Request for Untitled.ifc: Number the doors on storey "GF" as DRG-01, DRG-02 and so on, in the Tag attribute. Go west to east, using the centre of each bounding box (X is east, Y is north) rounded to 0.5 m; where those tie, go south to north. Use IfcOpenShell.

First a look at what the model holds.

```python
import ifcopenshell
import ifcopenshell.util.element
import ifcopenshell.util.placement

model = ifcopenshell.open("Untitled.ifc")
print(model.schema)
storey = next(s for s in model.by_type("IfcBuildingStorey") if s.Name == "GF")
doors = [e for e in ifcopenshell.util.element.get_decomposition(storey) if e.is_a("IfcDoor")]
for e in sorted(doors, key=lambda e: e.id()):
    origin = ifcopenshell.util.placement.get_local_placement(e.ObjectPlacement)[:3, 3]
    print(e.id(), e.Tag, e.Name, origin.round(2) + 0.0, sep=" | ")
```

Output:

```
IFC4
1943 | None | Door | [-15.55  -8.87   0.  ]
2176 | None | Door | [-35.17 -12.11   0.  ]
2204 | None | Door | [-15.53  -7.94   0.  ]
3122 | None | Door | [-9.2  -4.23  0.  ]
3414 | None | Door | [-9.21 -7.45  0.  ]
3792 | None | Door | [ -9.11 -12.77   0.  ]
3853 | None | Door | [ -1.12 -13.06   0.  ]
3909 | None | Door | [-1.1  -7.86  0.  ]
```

```python
import ifcopenshell
import ifcopenshell.geom
import ifcopenshell.util.element
import ifcopenshell.util.shape

model = ifcopenshell.open("Untitled.ifc")
settings = ifcopenshell.geom.settings()
settings.set("use-world-coords", True)


def centre(element):
    shape = ifcopenshell.geom.create_shape(settings, element)
    return ifcopenshell.util.shape.get_bbox_centroid(shape.geometry)


storey = next(s for s in model.by_type("IfcBuildingStorey") if s.Name == "GF")
doors = [e for e in ifcopenshell.util.element.get_decomposition(storey) if e.is_a("IfcDoor")]

# Insertion points can sit at a corner or the storey origin, so sort by the geometry (in metres).
centres = {e: centre(e) for e in doors}
doors.sort(key=lambda e: (round(centres[e][0] / 0.5), centres[e][1]))

for i, e in enumerate(doors, start=1):
    number = f"DRG-{i:02d}"
    e.Tag = number
    print(e.id(), number)

model.write("Untitled_edited.ifc")
```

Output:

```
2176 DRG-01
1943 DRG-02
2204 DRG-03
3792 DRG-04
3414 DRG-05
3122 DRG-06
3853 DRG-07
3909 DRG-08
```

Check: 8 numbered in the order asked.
